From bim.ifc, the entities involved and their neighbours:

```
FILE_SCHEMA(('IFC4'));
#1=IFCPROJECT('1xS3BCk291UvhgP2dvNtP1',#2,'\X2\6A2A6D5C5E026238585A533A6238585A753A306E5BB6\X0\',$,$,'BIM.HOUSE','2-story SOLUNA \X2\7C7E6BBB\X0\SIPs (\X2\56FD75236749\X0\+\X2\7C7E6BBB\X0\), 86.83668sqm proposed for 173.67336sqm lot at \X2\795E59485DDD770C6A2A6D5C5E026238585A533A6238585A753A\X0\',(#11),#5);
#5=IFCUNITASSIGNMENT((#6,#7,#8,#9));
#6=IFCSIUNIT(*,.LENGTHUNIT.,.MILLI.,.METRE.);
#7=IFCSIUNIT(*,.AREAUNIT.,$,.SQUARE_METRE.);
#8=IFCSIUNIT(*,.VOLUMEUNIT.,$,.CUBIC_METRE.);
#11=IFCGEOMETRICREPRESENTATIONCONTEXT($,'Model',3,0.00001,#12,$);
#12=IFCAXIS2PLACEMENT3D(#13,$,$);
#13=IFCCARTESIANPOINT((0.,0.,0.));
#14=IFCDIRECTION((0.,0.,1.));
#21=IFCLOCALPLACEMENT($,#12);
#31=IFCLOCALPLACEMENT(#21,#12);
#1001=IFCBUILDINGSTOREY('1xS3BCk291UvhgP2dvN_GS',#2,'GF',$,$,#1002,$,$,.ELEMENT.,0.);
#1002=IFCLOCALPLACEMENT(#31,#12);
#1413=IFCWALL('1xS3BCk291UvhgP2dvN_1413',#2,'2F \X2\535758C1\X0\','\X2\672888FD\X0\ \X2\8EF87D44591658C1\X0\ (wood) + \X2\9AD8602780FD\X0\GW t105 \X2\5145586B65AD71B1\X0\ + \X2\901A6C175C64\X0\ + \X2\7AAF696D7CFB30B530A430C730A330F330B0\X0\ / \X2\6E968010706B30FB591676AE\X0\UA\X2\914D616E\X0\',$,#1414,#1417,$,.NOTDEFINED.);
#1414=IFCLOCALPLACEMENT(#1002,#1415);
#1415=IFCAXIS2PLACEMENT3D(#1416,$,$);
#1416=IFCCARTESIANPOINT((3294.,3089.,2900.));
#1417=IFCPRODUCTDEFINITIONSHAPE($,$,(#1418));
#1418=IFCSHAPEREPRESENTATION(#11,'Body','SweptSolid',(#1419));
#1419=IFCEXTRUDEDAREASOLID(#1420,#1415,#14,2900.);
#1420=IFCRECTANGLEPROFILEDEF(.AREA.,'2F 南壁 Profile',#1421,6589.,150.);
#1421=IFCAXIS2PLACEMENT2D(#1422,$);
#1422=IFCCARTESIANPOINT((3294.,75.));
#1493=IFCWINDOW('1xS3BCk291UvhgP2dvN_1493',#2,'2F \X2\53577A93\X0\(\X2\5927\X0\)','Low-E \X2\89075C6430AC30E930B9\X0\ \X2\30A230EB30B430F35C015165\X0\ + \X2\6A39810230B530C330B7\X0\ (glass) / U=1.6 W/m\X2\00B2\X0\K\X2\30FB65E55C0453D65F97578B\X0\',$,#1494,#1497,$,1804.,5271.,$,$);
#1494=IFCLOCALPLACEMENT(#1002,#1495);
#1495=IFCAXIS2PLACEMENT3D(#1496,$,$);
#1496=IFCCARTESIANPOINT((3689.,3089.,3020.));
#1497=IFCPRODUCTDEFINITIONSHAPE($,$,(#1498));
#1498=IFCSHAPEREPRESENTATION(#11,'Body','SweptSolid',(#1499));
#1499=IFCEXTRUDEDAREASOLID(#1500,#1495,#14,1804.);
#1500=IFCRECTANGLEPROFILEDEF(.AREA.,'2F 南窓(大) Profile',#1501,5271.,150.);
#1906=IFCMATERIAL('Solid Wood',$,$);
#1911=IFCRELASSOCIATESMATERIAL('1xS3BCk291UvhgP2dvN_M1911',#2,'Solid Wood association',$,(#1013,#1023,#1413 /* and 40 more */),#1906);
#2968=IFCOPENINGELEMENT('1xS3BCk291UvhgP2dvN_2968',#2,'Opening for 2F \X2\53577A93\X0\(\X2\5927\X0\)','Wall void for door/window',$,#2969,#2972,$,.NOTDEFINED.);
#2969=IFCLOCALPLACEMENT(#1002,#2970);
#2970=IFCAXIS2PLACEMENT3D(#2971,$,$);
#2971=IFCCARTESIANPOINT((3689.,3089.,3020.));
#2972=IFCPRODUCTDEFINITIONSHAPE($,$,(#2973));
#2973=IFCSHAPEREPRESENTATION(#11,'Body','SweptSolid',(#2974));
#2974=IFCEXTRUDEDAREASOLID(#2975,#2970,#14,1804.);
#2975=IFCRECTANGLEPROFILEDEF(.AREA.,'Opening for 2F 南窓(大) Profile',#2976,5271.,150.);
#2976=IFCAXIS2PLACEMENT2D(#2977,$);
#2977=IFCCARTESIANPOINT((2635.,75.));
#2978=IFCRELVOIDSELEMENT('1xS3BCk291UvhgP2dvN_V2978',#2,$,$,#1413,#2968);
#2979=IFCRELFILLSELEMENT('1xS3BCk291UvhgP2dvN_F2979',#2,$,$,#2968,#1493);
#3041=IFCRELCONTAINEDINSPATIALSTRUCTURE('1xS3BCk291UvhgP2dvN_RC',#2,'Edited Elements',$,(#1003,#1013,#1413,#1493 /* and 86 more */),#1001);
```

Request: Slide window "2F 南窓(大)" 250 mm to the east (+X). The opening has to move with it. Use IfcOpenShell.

```python
import ifcopenshell
import ifcopenshell.api.geometry
import ifcopenshell.util.placement

model = ifcopenshell.open("bim.ifc")

window = model.by_guid("1xS3BCk291UvhgP2dvN_1493")
opening = window.FillsVoids[0].RelatingOpeningElement
wall = opening.VoidsElements[0].RelatingBuildingElement

wall_matrix = ifcopenshell.util.placement.get_local_placement(wall.ObjectPlacement)
shift = wall_matrix[:3, 0] * 250.0
before = ifcopenshell.util.placement.get_local_placement(window.ObjectPlacement)[:3, 3].copy()

# The window is not placed relative to its opening, so move both.
for product in (opening, window):
    matrix = ifcopenshell.util.placement.get_local_placement(product.ObjectPlacement)
    matrix[:3, 3] += shift
    ifcopenshell.api.geometry.edit_object_placement(model, product=product, matrix=matrix, is_si=False)

after = ifcopenshell.util.placement.get_local_placement(window.ObjectPlacement)[:3, 3]
print("window moved by", (after - before).round(3) + 0.0)

model.write("bim_rev.ifc")
```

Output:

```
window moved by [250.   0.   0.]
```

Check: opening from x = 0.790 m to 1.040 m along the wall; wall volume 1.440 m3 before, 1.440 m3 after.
